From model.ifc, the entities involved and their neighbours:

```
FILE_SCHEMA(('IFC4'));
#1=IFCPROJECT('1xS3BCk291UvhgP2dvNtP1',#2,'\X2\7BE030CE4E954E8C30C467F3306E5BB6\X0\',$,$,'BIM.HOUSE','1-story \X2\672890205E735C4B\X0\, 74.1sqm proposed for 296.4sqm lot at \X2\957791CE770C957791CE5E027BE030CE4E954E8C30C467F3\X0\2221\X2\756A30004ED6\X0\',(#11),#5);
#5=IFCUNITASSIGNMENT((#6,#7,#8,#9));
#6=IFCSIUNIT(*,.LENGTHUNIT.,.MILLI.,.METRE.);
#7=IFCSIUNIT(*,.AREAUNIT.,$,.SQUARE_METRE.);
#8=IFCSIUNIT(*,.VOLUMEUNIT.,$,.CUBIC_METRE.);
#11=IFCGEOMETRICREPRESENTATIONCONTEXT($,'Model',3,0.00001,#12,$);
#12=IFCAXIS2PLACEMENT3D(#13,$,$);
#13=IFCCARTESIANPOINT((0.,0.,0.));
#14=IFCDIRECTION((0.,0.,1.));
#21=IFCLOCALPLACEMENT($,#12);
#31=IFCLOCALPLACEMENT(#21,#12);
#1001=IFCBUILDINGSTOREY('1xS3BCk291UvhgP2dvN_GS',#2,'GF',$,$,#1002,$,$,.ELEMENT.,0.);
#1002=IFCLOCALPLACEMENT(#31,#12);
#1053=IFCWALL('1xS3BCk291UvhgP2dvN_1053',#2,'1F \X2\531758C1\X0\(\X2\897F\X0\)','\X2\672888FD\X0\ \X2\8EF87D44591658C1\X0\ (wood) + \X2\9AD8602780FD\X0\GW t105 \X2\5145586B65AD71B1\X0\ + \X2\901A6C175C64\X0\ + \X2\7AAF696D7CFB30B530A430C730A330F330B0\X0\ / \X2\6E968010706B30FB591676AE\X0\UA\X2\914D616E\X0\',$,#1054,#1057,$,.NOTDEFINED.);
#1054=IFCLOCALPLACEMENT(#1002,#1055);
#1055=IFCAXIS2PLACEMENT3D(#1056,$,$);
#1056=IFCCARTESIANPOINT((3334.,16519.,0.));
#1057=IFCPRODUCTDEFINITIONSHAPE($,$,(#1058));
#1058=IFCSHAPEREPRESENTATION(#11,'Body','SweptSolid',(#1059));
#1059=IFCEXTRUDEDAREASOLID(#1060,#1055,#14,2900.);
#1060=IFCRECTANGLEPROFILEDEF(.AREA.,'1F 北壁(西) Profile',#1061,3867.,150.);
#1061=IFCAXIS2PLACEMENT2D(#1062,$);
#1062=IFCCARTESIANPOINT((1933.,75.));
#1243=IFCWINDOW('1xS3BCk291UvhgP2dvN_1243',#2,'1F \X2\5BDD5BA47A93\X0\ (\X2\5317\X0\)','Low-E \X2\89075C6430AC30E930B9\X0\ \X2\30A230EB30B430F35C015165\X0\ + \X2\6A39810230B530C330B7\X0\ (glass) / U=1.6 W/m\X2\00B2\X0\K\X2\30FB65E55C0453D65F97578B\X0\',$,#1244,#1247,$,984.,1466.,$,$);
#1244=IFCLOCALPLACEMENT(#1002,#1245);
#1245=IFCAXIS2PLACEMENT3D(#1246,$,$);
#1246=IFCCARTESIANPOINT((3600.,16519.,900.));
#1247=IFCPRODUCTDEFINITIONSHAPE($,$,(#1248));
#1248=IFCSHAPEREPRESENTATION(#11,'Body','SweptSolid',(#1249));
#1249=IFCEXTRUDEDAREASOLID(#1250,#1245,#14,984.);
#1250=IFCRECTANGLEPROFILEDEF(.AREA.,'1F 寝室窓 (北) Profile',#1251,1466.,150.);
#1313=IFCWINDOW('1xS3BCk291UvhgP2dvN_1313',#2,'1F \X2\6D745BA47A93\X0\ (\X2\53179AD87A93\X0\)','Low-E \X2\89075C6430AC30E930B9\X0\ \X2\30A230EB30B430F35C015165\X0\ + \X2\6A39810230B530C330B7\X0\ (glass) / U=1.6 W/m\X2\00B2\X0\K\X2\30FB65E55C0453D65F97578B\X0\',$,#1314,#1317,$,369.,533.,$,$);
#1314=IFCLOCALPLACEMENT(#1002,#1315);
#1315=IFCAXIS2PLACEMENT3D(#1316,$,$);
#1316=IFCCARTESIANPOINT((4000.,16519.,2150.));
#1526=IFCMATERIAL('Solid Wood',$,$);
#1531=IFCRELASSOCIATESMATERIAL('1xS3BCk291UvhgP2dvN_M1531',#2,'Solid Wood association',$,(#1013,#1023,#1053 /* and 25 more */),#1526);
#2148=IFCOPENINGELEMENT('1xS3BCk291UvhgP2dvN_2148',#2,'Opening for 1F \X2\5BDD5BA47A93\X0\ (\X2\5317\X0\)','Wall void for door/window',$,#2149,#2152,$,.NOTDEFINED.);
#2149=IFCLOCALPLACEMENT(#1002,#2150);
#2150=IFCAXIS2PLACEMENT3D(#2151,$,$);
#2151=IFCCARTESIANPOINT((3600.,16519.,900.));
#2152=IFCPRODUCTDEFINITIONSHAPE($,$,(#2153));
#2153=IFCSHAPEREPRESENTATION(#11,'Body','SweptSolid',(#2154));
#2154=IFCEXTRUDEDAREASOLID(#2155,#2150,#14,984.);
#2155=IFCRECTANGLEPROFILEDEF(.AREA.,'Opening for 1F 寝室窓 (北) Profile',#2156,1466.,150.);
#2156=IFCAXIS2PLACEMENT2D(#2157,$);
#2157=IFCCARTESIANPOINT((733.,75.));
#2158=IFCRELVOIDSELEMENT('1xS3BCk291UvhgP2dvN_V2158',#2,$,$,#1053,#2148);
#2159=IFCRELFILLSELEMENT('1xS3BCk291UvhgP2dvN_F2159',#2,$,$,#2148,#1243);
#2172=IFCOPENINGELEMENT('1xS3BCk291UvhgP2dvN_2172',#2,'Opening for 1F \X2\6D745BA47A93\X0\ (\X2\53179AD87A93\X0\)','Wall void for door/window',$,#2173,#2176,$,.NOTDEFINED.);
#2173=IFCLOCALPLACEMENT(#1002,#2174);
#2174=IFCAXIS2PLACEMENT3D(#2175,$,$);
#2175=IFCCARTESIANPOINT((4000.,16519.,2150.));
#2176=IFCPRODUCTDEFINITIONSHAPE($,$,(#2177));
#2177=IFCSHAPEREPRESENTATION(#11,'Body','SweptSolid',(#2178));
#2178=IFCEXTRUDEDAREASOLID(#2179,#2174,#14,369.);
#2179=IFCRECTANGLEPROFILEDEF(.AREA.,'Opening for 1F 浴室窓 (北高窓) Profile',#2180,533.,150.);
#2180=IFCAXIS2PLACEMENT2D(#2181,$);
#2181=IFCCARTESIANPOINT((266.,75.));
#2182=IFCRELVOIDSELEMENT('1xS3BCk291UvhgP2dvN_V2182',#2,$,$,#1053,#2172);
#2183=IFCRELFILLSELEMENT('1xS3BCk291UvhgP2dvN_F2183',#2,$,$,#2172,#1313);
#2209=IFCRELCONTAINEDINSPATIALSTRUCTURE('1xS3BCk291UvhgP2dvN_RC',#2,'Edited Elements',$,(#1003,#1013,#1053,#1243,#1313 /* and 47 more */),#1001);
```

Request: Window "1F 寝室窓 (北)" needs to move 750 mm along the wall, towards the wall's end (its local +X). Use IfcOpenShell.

```python
import ifcopenshell
import ifcopenshell.api.geometry
import ifcopenshell.util.placement
import ifcopenshell.util.unit

model = ifcopenshell.open("model.ifc")
unit_scale = ifcopenshell.util.unit.calculate_unit_scale(model)

window = model.by_id(1243)
opening = window.FillsVoids[0].RelatingOpeningElement
wall = opening.VoidsElements[0].RelatingBuildingElement

wall_matrix = ifcopenshell.util.placement.get_local_placement(wall.ObjectPlacement)
shift = wall_matrix[:3, 0] * 0.75 / unit_scale
before = ifcopenshell.util.placement.get_local_placement(window.ObjectPlacement)[:3, 3].copy()

# The window is not placed relative to its opening, so move both.
for product in (opening, window):
    matrix = ifcopenshell.util.placement.get_local_placement(product.ObjectPlacement)
    matrix[:3, 3] += shift
    ifcopenshell.api.geometry.edit_object_placement(model, product=product, matrix=matrix, is_si=False)

after = ifcopenshell.util.placement.get_local_placement(window.ObjectPlacement)[:3, 3]
print("window moved by", (after - before).round(3) + 0.0)

model.write("model-out.ifc")
```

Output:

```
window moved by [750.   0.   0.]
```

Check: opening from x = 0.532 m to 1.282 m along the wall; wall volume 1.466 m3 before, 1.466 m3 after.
